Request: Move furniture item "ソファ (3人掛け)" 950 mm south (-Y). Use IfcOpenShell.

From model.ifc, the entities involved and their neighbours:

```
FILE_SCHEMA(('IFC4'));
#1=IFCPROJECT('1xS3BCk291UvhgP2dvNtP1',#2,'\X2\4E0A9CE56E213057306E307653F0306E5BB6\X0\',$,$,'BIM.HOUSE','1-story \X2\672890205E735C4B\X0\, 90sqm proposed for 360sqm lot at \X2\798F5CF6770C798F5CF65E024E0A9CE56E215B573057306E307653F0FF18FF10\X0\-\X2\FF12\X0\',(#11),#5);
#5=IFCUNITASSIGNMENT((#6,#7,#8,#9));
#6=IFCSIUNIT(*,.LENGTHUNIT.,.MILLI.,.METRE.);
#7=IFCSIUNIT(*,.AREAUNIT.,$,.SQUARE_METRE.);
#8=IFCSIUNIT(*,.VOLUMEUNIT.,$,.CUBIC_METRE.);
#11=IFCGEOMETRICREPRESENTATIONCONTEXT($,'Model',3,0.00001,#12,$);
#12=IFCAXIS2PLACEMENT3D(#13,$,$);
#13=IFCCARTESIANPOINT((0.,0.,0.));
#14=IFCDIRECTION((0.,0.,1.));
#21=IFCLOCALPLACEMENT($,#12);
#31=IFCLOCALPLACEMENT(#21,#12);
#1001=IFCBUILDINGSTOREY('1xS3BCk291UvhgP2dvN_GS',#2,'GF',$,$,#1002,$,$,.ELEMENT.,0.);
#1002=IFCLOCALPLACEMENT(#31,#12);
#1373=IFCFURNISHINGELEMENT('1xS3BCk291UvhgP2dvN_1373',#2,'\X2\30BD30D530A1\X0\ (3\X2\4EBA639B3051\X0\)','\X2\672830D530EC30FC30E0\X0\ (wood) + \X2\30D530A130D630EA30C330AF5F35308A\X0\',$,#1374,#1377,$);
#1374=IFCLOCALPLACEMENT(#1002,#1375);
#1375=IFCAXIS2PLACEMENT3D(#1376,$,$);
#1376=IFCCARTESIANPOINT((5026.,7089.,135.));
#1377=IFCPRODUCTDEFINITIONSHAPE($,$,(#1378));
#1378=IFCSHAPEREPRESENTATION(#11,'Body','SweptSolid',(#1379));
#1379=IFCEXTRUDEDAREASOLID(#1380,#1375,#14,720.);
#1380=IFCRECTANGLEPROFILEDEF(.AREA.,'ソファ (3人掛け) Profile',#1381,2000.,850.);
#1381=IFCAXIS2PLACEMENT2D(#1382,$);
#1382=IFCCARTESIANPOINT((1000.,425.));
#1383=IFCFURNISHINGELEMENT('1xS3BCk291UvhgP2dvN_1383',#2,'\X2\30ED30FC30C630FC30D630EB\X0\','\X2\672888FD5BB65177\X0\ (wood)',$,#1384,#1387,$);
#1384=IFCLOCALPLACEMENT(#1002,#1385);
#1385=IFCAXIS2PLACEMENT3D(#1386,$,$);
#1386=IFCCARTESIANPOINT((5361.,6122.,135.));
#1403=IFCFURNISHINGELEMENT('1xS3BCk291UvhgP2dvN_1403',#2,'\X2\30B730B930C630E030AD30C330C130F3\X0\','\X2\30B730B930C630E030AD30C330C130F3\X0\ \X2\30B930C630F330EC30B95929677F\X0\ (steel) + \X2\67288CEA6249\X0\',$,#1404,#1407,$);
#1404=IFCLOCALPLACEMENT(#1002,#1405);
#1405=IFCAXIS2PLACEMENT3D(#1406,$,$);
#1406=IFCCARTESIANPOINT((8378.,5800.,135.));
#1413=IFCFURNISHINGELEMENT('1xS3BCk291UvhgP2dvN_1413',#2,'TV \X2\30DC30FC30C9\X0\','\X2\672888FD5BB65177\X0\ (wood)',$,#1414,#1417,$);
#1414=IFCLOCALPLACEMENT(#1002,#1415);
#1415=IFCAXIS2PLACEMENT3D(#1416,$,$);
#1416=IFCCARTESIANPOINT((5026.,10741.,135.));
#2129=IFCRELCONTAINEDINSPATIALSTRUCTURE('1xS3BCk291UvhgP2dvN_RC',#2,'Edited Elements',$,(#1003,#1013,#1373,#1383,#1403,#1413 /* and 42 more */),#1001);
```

```python
import ifcopenshell
import ifcopenshell.api.geometry
import ifcopenshell.util.placement
import ifcopenshell.util.unit

model = ifcopenshell.open("model.ifc")
unit_scale = ifcopenshell.util.unit.calculate_unit_scale(model)

item = model.by_guid("1xS3BCk291UvhgP2dvN_1373")
matrix = ifcopenshell.util.placement.get_local_placement(item.ObjectPlacement)
matrix[1, 3] -= 0.95 / unit_scale
ifcopenshell.api.geometry.edit_object_placement(model, product=item, matrix=matrix, is_si=False)

print(ifcopenshell.util.placement.get_local_placement(item.ObjectPlacement).round(3) + 0.0)

model.write("model-out.ifc")
```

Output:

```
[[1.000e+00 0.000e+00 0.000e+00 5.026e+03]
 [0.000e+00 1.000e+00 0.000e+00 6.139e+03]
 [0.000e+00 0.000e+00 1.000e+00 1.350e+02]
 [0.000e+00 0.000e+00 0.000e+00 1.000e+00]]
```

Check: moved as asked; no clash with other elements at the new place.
